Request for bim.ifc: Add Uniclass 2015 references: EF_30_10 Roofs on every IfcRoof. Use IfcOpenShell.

First a look at what the model holds.

```python
import ifcopenshell

model = ifcopenshell.open("bim.ifc")
print(model.schema)
print("classifications:", [c.Name for c in model.by_type("IfcClassification")])
for ifc_class in ("IfcDoor", "IfcRoof", "IfcStair", "IfcWall", "IfcWindow"):
    print(ifc_class, len(model.by_type(ifc_class)))
```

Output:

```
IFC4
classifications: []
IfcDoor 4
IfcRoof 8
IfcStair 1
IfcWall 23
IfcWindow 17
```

```python
import ifcopenshell
import ifcopenshell.api.classification

model = ifcopenshell.open("bim.ifc")

system = ifcopenshell.api.classification.add_classification(model, classification="Uniclass 2015")

codes = {
    "IfcRoof": ("EF_30_10", "Roofs"),
}
for ifc_class, (code, name) in codes.items():
    products = model.by_type(ifc_class)
    ifcopenshell.api.classification.add_reference(
        model, products=products, classification=system, identification=code, name=name
    )
    print(code, len(products))

model.write("bim_v2.ifc")
```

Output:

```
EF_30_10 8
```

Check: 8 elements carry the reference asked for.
